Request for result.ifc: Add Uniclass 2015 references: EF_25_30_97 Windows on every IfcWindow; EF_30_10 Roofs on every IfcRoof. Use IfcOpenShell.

First a look at what the model holds.

```python
import ifcopenshell

model = ifcopenshell.open("result.ifc")
print(model.schema)
print("classifications:", [c.Name for c in model.by_type("IfcClassification")])
for ifc_class in ("IfcDoor", "IfcRoof", "IfcStair", "IfcWall", "IfcWindow"):
    print(ifc_class, len(model.by_type(ifc_class)))
```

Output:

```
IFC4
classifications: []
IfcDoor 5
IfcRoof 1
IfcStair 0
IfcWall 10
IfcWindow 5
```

```python
import ifcopenshell
import ifcopenshell.api.classification

model = ifcopenshell.open("result.ifc")

system = ifcopenshell.api.classification.add_classification(model, classification="Uniclass 2015")

codes = {
    "IfcWindow": ("EF_25_30_97", "Windows"),
    "IfcRoof": ("EF_30_10", "Roofs"),
}
for ifc_class, (code, name) in codes.items():
    products = model.by_type(ifc_class)
    ifcopenshell.api.classification.add_reference(
        model, products=products, classification=system, identification=code, name=name
    )
    print(code, len(products))

model.write("result_edited.ifc")
```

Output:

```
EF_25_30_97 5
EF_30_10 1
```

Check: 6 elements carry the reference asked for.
